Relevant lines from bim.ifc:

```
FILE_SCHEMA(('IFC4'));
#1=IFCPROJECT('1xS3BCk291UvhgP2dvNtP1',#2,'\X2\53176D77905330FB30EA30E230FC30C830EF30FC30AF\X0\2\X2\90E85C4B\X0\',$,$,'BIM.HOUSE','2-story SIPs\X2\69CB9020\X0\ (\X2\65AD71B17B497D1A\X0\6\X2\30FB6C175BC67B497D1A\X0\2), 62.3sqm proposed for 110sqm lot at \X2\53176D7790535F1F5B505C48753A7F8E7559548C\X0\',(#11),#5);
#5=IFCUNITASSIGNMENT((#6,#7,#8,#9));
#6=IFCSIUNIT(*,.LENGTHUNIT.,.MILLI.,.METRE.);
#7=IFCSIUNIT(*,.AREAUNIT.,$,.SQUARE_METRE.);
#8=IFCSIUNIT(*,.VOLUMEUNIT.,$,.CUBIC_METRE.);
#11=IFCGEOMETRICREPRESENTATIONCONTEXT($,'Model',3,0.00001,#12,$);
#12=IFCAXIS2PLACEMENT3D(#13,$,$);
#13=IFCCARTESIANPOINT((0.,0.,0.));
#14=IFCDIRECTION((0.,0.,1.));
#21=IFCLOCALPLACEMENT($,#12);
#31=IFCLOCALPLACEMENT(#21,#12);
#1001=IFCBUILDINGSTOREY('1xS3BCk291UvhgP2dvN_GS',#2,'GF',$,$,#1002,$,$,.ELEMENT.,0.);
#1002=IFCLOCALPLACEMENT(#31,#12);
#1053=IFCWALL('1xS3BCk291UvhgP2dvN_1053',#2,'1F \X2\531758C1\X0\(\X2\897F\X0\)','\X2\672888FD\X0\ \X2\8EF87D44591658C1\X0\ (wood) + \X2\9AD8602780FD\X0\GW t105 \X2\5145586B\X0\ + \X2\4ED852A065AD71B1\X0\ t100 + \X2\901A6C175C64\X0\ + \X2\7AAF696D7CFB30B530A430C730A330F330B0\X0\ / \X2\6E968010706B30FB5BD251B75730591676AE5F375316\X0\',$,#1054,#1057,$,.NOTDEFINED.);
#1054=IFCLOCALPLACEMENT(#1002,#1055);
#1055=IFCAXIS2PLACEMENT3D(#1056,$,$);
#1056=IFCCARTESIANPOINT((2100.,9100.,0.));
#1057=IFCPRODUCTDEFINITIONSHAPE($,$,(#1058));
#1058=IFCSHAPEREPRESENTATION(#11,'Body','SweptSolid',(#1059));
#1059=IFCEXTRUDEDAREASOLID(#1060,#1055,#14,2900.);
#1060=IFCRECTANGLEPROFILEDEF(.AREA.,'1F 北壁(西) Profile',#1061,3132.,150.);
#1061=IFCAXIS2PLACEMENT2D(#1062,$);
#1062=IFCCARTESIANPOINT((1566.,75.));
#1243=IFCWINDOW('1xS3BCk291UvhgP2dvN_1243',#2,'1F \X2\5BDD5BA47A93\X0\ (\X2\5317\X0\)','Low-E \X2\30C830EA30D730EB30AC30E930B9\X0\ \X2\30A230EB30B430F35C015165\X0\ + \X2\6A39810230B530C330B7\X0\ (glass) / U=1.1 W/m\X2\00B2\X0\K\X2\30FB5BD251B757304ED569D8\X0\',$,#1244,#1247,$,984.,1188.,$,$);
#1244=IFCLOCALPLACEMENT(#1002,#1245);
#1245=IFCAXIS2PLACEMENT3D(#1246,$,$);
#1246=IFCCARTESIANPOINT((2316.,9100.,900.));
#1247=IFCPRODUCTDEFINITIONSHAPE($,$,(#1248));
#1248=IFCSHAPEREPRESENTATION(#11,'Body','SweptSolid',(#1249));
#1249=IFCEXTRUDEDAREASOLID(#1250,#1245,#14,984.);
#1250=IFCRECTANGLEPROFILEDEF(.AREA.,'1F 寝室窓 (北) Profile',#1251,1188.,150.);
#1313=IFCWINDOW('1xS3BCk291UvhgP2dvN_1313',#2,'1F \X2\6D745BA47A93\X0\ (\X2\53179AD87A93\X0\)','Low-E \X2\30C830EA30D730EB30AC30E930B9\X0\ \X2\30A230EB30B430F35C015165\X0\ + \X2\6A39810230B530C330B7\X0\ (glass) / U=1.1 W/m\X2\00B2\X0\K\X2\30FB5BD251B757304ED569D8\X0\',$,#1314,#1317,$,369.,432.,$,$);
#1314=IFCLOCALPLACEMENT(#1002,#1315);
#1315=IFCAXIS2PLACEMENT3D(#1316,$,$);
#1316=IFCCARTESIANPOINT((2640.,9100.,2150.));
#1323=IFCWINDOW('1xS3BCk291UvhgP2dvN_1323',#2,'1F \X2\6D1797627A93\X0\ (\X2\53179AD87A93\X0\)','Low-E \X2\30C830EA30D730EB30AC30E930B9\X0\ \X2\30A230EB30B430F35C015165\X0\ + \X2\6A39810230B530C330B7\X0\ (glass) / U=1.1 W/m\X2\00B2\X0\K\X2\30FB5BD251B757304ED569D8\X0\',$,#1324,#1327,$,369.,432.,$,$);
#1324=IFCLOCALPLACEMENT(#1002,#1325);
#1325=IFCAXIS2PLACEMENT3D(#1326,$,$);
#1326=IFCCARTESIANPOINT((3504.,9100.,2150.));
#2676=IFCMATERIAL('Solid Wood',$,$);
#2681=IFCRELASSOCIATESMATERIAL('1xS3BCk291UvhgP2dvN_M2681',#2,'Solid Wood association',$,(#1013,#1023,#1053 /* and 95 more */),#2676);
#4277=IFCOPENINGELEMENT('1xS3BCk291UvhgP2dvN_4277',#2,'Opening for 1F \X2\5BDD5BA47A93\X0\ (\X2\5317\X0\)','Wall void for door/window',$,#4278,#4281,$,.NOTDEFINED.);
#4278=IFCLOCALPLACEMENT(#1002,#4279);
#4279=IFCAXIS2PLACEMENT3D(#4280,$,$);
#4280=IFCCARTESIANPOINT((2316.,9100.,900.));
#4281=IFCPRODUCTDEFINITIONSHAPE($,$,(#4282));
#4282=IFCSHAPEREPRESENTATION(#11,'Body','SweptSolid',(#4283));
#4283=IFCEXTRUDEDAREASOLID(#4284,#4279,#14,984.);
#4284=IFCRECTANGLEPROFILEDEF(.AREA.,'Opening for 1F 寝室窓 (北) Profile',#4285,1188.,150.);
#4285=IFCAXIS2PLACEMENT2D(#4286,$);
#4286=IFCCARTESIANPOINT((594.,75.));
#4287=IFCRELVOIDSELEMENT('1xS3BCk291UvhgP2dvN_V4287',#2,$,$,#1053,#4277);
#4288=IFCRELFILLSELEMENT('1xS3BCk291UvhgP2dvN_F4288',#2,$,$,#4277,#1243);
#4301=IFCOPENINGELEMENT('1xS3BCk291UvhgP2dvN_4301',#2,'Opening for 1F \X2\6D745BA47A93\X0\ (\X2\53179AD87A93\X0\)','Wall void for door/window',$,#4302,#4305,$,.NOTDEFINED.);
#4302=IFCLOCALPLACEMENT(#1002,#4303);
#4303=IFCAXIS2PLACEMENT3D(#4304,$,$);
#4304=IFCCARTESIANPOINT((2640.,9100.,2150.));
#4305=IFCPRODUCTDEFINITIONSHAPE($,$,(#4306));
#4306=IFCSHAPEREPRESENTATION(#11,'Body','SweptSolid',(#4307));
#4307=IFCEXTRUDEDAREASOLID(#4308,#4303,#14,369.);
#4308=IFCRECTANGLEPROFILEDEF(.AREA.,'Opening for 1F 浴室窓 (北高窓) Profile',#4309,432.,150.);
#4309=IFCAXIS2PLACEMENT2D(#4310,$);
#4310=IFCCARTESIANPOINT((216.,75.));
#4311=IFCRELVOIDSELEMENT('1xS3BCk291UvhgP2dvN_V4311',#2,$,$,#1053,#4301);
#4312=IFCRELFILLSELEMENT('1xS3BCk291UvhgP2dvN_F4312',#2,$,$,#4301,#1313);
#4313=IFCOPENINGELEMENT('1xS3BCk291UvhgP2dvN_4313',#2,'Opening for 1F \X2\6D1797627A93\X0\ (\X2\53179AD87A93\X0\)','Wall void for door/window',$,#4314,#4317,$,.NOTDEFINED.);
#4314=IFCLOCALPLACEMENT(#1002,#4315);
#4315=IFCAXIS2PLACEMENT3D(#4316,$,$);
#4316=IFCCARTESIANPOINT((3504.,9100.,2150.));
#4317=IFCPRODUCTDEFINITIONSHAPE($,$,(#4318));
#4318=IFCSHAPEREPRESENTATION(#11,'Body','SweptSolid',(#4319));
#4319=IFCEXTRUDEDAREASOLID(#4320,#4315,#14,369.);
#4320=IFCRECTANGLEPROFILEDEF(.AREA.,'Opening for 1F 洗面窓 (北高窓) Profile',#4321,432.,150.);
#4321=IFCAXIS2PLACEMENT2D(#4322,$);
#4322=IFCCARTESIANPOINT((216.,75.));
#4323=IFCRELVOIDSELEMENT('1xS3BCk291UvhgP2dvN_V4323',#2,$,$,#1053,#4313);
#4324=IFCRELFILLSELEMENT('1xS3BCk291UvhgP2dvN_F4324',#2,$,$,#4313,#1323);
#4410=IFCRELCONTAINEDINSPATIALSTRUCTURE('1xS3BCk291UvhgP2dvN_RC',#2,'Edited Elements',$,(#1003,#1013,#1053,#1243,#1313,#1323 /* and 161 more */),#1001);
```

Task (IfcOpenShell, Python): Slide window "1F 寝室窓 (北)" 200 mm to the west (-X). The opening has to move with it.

```python
import ifcopenshell
import ifcopenshell.api.geometry
import ifcopenshell.util.placement
import ifcopenshell.util.unit

model = ifcopenshell.open("bim.ifc")
unit_scale = ifcopenshell.util.unit.calculate_unit_scale(model)

window = model.by_guid("1xS3BCk291UvhgP2dvN_1243")
opening = window.FillsVoids[0].RelatingOpeningElement
wall = opening.VoidsElements[0].RelatingBuildingElement

wall_matrix = ifcopenshell.util.placement.get_local_placement(wall.ObjectPlacement)
shift = wall_matrix[:3, 0] * -0.2 / unit_scale
before = ifcopenshell.util.placement.get_local_placement(window.ObjectPlacement)[:3, 3].copy()

# The window is not placed relative to its opening, so move both.
for product in (opening, window):
    matrix = ifcopenshell.util.placement.get_local_placement(product.ObjectPlacement)
    matrix[:3, 3] += shift
    ifcopenshell.api.geometry.edit_object_placement(model, product=product, matrix=matrix, is_si=False)

after = ifcopenshell.util.placement.get_local_placement(window.ObjectPlacement)[:3, 3]
print("window moved by", (after - before).round(3) + 0.0)

model.write("bim_edited.ifc")
```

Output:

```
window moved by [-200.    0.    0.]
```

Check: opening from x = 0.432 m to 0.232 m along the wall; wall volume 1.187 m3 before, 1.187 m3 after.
